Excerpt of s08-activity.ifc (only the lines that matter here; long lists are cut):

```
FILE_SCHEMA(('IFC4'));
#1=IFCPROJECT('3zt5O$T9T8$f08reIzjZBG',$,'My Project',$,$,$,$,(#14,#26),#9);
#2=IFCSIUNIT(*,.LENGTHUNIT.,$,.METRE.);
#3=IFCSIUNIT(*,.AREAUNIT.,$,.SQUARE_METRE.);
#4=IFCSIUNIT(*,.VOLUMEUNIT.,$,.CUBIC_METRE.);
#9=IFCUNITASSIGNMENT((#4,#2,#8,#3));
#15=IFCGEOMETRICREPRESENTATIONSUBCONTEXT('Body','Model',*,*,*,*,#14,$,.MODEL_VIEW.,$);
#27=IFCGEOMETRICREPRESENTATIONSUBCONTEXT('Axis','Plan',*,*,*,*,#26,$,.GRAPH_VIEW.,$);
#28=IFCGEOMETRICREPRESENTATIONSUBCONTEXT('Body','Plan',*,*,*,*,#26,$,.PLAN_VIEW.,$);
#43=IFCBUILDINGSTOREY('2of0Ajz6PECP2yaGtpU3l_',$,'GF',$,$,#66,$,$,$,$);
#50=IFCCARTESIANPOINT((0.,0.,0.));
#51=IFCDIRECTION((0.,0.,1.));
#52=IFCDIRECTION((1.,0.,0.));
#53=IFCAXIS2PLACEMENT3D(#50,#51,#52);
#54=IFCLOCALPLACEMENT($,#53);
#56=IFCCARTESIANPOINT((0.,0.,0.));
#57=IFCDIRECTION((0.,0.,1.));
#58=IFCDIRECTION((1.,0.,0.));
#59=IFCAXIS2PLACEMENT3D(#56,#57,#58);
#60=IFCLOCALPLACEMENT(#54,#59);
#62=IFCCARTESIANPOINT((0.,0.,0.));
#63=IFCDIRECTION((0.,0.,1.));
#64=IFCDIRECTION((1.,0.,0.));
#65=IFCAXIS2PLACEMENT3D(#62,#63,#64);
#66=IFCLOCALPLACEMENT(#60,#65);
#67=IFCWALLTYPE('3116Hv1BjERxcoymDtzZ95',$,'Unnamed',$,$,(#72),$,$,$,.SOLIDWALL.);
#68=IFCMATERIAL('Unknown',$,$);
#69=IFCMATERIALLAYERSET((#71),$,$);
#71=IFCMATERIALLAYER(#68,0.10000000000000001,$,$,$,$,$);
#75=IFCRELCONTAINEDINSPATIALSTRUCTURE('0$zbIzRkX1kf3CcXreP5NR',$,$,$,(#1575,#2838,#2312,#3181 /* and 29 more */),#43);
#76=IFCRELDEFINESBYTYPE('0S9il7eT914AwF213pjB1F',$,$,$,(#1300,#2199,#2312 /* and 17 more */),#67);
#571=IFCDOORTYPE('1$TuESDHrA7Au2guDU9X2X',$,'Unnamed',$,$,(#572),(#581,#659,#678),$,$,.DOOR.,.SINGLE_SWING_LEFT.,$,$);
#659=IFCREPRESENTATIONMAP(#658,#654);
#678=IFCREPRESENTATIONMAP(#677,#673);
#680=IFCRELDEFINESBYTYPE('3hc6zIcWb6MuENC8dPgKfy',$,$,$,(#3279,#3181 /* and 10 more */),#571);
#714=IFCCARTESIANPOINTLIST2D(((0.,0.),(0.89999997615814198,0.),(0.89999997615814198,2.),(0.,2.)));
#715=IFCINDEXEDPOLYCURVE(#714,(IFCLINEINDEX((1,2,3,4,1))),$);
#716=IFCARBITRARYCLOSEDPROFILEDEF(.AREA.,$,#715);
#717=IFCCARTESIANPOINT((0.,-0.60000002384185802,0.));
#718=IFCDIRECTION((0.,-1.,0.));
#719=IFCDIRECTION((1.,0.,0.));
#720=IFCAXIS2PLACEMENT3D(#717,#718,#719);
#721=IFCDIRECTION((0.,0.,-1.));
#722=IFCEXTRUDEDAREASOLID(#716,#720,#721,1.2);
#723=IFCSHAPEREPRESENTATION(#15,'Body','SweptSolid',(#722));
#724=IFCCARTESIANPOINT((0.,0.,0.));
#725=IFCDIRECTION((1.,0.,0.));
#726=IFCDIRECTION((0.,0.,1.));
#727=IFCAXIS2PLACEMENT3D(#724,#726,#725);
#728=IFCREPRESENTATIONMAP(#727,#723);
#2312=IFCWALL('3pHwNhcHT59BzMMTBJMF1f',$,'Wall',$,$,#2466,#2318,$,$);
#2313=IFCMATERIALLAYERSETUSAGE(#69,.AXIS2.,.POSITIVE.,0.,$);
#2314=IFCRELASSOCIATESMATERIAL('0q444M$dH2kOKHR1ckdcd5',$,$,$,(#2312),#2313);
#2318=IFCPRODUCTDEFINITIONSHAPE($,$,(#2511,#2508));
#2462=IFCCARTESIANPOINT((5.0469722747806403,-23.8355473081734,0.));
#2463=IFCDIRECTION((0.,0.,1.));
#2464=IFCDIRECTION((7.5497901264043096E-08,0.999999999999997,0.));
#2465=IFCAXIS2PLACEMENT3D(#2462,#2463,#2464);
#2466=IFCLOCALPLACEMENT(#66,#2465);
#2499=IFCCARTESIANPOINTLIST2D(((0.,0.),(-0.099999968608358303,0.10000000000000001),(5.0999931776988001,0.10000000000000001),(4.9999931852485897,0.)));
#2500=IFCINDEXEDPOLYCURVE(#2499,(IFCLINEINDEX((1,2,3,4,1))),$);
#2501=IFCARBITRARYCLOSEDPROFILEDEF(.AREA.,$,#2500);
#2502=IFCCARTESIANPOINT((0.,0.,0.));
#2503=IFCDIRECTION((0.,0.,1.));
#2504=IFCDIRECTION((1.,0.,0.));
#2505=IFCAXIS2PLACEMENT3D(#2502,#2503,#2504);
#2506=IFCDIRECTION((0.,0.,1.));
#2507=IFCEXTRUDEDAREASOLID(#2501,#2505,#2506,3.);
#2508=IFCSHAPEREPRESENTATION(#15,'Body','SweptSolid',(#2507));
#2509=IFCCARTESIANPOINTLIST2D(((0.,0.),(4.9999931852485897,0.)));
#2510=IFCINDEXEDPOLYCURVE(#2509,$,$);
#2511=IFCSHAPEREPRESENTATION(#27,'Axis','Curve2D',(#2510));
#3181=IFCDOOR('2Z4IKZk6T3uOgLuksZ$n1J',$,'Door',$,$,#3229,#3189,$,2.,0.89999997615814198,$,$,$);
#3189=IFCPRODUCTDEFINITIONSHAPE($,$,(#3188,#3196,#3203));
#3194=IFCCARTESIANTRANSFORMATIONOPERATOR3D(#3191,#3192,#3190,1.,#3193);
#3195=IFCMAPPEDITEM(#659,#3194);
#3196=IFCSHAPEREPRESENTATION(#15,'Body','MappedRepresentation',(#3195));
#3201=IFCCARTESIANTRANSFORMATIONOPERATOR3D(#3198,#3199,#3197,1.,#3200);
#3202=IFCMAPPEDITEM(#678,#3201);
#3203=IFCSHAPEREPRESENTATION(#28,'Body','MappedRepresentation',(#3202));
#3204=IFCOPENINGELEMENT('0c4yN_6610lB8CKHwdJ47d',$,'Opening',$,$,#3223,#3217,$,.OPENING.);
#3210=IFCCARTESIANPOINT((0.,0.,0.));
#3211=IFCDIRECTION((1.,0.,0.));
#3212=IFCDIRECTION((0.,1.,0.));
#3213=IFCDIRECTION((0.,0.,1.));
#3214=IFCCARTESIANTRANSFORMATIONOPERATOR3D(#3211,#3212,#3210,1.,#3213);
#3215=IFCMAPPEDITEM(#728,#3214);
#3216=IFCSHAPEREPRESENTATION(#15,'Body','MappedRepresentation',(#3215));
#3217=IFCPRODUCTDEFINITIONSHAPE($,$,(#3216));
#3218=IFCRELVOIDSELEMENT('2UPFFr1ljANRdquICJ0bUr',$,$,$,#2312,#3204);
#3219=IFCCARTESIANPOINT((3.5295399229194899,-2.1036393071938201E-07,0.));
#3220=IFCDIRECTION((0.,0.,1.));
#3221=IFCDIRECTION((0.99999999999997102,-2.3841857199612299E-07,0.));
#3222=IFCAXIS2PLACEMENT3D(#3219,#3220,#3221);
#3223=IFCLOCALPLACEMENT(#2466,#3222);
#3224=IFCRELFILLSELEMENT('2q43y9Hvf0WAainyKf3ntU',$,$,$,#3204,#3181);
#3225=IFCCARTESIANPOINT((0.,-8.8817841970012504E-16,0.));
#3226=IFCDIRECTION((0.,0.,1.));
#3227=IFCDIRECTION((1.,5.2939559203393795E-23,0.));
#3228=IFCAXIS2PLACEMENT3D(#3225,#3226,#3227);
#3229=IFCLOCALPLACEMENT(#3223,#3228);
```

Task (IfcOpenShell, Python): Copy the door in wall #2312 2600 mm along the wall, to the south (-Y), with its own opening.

```python
import ifcopenshell
import ifcopenshell.api.feature
import ifcopenshell.api.geometry
import ifcopenshell.api.root
import ifcopenshell.geom
import ifcopenshell.util.element
import ifcopenshell.util.placement
import ifcopenshell.util.shape
import ifcopenshell.util.unit

model = ifcopenshell.open("s08-activity.ifc")
unit_scale = ifcopenshell.util.unit.calculate_unit_scale(model)
settings = ifcopenshell.geom.settings()


def volume(element):
    """Net volume in cubic metres, openings subtracted."""
    shape = ifcopenshell.geom.create_shape(settings, element)
    return ifcopenshell.util.shape.get_volume(shape.geometry)


door = model.by_guid("2Z4IKZk6T3uOgLuksZ$n1J")
opening = door.FillsVoids[0].RelatingOpeningElement
wall = opening.VoidsElements[0].RelatingBuildingElement
before = volume(wall)
shift = ifcopenshell.util.placement.get_local_placement(wall.ObjectPlacement)[:3, 0] * -2.6 / unit_scale

# copy_class copies the void relationship, type, container and properties, but no geometry.
new_opening = ifcopenshell.api.root.copy_class(model, product=opening)
new_opening.Representation = ifcopenshell.util.element.copy_deep(
    model, opening.Representation, exclude=["IfcGeometricRepresentationContext", "IfcRepresentationMap"]
)
new_door = ifcopenshell.api.root.copy_class(model, product=door)
new_door.Representation = ifcopenshell.util.element.copy_deep(
    model, door.Representation, exclude=["IfcGeometricRepresentationContext", "IfcRepresentationMap"]
)
ifcopenshell.api.feature.add_filling(model, opening=new_opening, element=new_door)

for old, new in ((opening, new_opening), (door, new_door)):
    matrix = ifcopenshell.util.placement.get_local_placement(old.ObjectPlacement)
    matrix[:3, 3] += shift
    ifcopenshell.api.geometry.edit_object_placement(model, product=new, matrix=matrix, is_si=False)

after = volume(wall)

print(f"wall volume {before:.3f} -> {after:.3f} m3")

model.write("s08-activity_rev.ifc")
```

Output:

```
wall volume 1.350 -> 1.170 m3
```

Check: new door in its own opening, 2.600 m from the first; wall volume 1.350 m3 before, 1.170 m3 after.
